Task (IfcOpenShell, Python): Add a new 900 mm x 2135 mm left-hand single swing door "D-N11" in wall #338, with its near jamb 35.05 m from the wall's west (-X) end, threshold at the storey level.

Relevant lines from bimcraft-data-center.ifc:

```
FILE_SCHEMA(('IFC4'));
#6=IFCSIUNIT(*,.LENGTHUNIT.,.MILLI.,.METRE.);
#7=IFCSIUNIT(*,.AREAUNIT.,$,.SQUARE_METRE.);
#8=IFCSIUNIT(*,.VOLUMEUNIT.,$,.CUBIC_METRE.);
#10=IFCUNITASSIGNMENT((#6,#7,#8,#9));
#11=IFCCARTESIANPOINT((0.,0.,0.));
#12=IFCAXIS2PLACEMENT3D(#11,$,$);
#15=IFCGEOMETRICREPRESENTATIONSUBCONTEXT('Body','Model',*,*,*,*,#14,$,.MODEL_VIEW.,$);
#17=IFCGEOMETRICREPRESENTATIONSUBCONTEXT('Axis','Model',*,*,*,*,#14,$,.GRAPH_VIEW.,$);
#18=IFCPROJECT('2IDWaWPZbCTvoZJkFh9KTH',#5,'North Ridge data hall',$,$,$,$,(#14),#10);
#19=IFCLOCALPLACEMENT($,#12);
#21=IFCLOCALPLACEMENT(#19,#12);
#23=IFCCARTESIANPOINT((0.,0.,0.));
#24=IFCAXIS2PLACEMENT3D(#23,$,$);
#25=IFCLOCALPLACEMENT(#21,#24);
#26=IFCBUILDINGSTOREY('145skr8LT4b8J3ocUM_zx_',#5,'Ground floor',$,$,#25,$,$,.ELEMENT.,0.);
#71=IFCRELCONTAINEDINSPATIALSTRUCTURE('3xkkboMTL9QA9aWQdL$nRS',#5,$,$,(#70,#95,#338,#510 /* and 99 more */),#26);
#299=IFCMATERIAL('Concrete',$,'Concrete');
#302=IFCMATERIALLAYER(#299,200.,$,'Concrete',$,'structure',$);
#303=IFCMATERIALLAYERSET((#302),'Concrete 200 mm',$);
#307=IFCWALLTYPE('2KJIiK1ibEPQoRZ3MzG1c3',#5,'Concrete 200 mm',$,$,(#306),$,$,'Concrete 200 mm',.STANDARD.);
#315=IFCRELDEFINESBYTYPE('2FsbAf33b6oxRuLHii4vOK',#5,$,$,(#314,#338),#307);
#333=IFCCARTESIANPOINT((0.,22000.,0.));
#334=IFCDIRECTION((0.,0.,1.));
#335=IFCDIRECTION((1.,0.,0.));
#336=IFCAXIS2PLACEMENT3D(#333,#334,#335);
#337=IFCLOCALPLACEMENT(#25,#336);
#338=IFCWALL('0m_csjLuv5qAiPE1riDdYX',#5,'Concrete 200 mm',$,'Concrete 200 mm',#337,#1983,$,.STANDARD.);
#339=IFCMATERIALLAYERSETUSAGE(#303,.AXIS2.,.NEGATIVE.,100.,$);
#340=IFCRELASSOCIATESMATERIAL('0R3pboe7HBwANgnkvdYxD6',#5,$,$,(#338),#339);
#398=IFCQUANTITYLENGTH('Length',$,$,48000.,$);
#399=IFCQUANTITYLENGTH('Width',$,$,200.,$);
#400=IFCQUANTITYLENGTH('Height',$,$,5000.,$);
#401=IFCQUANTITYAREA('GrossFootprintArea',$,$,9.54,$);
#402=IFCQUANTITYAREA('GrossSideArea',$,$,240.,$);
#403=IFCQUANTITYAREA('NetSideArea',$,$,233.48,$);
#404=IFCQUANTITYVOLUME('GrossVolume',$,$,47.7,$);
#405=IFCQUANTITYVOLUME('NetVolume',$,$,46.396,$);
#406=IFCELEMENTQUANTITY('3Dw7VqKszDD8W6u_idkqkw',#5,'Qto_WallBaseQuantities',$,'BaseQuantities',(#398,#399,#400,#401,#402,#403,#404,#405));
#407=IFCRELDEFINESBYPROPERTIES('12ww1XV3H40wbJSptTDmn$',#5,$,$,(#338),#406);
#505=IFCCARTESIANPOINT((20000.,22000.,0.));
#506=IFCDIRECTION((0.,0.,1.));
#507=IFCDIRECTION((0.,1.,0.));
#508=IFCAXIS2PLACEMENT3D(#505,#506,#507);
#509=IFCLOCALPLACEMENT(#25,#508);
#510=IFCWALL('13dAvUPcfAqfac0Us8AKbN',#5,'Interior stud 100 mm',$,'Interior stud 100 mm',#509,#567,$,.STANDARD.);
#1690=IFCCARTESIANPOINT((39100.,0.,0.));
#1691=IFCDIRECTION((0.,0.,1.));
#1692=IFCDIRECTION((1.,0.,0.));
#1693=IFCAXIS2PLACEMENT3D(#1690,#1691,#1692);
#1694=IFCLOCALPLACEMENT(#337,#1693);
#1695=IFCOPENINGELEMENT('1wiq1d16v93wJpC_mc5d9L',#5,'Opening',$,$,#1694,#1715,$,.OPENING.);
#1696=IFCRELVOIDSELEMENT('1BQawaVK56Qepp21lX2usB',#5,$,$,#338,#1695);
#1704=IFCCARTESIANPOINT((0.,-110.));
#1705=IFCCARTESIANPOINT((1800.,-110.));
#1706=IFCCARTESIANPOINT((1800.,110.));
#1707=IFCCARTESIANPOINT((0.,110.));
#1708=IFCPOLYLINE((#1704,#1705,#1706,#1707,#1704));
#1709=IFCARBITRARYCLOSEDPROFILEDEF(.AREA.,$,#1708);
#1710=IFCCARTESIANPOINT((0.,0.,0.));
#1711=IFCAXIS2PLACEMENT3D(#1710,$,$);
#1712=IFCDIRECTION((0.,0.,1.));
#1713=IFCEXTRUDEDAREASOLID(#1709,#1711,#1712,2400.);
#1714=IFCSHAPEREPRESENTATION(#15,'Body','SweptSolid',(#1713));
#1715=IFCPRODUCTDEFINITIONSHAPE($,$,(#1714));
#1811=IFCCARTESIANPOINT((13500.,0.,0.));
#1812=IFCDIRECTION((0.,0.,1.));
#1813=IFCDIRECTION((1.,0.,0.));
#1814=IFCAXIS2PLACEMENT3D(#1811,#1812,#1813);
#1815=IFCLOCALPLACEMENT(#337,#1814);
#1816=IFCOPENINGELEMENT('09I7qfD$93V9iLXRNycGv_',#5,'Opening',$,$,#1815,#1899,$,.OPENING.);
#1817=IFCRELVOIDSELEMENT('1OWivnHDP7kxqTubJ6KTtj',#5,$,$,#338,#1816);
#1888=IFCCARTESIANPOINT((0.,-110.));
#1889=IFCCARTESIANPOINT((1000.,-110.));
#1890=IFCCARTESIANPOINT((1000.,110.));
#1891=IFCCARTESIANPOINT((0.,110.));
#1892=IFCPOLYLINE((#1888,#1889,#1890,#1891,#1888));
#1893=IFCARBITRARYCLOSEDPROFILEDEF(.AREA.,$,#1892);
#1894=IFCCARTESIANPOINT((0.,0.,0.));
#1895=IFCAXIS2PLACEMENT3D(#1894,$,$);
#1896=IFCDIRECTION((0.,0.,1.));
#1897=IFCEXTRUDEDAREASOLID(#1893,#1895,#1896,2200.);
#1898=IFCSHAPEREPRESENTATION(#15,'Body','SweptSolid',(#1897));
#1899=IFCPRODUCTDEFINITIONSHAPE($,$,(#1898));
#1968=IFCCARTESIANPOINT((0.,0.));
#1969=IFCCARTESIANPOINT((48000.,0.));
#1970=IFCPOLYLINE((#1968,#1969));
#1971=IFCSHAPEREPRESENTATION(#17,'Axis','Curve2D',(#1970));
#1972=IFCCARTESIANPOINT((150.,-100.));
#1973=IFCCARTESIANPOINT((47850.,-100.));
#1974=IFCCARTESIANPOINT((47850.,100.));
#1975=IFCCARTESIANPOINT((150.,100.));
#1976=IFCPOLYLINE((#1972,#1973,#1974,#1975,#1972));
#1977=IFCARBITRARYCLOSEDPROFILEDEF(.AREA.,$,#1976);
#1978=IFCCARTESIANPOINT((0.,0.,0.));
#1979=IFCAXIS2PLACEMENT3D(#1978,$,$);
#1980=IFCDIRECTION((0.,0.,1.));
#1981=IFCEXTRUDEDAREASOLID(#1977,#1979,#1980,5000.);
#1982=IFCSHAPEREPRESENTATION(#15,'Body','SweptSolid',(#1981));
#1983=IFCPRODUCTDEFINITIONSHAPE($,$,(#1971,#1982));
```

```python
import numpy as np
import ifcopenshell
import ifcopenshell.api.feature
import ifcopenshell.api.geometry
import ifcopenshell.api.pset
import ifcopenshell.api.root
import ifcopenshell.api.spatial
import ifcopenshell.geom
import ifcopenshell.util.element
import ifcopenshell.util.placement
import ifcopenshell.util.representation
import ifcopenshell.util.shape
import ifcopenshell.util.unit

model = ifcopenshell.open("bimcraft-data-center.ifc")
unit_scale = ifcopenshell.util.unit.calculate_unit_scale(model)
area_scale = ifcopenshell.util.unit.calculate_unit_scale(model, "AREAUNIT")
volume_scale = ifcopenshell.util.unit.calculate_unit_scale(model, "VOLUMEUNIT")
settings = ifcopenshell.geom.settings()


def volume(element):
    """Net volume in cubic metres, openings subtracted."""
    shape = ifcopenshell.geom.create_shape(settings, element)
    return ifcopenshell.util.shape.get_volume(shape.geometry)


wall = model.by_guid("0m_csjLuv5qAiPE1riDdYX")
storey = ifcopenshell.util.element.get_container(wall, ifc_class="IfcBuildingStorey")
context = ifcopenshell.util.representation.get_context(model, "Model", "Body", "MODEL_VIEW")
before = volume(wall)

width, height, from_end, sill = 0.9, 2.135, 35.05, 0.0  # metres

# The wall runs along its own X axis, and the end named is its -X end.
wall_shape = ifcopenshell.geom.create_shape(settings, wall)
x, y, z = ifcopenshell.util.shape.get_vertices(wall_shape.geometry).T
start = x.min() + from_end
face, thickness = float(y.min()), float(y.max() - y.min())
wall_matrix = ifcopenshell.util.placement.get_local_placement(wall.ObjectPlacement)
level = ifcopenshell.util.placement.get_local_placement(storey.ObjectPlacement)[2, 3]


def in_wall(x, y):
    """Placement at x, y metres in the wall's axes, at sill height."""
    matrix = wall_matrix.copy()
    matrix[:, 3] = wall_matrix @ np.array([x / unit_scale, y / unit_scale, 0.0, 1.0])
    matrix[2, 3] = level + sill / unit_scale
    return matrix


# Opening: a box that overshoots both wall faces by 50 mm.
opening = ifcopenshell.api.root.create_entity(model, ifc_class="IfcOpeningElement", predefined_type="OPENING")
box = ifcopenshell.api.geometry.add_wall_representation(
    model, context=context, length=width, height=height, thickness=thickness + 0.1
)
ifcopenshell.api.geometry.assign_representation(model, product=opening, representation=box)
ifcopenshell.api.geometry.edit_object_placement(model, product=opening, matrix=in_wall(start, face - 0.05), is_si=False)
ifcopenshell.api.feature.add_feature(model, feature=opening, element=wall)

door = ifcopenshell.api.root.create_entity(model, ifc_class="IfcDoor", name="D-N11", predefined_type="DOOR")
door.OverallWidth, door.OverallHeight = width / unit_scale, height / unit_scale
door.OperationType = "SINGLE_SWING_LEFT"
body = ifcopenshell.api.geometry.add_door_representation(
    model,
    context=context,
    overall_width=door.OverallWidth,
    overall_height=door.OverallHeight,
    operation_type="SINGLE_SWING_LEFT",
    lining_properties={"LiningDepth": thickness / unit_scale, "ThresholdDepth": thickness / unit_scale},
)
ifcopenshell.api.geometry.assign_representation(model, product=door, representation=body)
ifcopenshell.api.spatial.assign_container(model, products=[door], relating_structure=storey)
ifcopenshell.api.feature.add_filling(model, opening=opening, element=door)

# The lining spans the wall, so the door starts at the wall face.
ifcopenshell.api.geometry.edit_object_placement(model, product=door, matrix=in_wall(start, face), is_si=False)

after = volume(wall)

# Update the wall's stored quantities.
qto = model.by_id(ifcopenshell.util.element.get_pset(wall, "Qto_WallBaseQuantities", should_inherit=False)["id"])
ifcopenshell.api.pset.edit_qto(model, qto=qto, properties={
    "NetSideArea": after / thickness / area_scale,
    "NetVolume": after / volume_scale,
})

print(f"wall volume {before:.3f} -> {after:.3f} m3")

model.write("bimcraft-data-center_rev.ifc")
```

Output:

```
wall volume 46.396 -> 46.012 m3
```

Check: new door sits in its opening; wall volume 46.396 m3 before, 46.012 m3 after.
